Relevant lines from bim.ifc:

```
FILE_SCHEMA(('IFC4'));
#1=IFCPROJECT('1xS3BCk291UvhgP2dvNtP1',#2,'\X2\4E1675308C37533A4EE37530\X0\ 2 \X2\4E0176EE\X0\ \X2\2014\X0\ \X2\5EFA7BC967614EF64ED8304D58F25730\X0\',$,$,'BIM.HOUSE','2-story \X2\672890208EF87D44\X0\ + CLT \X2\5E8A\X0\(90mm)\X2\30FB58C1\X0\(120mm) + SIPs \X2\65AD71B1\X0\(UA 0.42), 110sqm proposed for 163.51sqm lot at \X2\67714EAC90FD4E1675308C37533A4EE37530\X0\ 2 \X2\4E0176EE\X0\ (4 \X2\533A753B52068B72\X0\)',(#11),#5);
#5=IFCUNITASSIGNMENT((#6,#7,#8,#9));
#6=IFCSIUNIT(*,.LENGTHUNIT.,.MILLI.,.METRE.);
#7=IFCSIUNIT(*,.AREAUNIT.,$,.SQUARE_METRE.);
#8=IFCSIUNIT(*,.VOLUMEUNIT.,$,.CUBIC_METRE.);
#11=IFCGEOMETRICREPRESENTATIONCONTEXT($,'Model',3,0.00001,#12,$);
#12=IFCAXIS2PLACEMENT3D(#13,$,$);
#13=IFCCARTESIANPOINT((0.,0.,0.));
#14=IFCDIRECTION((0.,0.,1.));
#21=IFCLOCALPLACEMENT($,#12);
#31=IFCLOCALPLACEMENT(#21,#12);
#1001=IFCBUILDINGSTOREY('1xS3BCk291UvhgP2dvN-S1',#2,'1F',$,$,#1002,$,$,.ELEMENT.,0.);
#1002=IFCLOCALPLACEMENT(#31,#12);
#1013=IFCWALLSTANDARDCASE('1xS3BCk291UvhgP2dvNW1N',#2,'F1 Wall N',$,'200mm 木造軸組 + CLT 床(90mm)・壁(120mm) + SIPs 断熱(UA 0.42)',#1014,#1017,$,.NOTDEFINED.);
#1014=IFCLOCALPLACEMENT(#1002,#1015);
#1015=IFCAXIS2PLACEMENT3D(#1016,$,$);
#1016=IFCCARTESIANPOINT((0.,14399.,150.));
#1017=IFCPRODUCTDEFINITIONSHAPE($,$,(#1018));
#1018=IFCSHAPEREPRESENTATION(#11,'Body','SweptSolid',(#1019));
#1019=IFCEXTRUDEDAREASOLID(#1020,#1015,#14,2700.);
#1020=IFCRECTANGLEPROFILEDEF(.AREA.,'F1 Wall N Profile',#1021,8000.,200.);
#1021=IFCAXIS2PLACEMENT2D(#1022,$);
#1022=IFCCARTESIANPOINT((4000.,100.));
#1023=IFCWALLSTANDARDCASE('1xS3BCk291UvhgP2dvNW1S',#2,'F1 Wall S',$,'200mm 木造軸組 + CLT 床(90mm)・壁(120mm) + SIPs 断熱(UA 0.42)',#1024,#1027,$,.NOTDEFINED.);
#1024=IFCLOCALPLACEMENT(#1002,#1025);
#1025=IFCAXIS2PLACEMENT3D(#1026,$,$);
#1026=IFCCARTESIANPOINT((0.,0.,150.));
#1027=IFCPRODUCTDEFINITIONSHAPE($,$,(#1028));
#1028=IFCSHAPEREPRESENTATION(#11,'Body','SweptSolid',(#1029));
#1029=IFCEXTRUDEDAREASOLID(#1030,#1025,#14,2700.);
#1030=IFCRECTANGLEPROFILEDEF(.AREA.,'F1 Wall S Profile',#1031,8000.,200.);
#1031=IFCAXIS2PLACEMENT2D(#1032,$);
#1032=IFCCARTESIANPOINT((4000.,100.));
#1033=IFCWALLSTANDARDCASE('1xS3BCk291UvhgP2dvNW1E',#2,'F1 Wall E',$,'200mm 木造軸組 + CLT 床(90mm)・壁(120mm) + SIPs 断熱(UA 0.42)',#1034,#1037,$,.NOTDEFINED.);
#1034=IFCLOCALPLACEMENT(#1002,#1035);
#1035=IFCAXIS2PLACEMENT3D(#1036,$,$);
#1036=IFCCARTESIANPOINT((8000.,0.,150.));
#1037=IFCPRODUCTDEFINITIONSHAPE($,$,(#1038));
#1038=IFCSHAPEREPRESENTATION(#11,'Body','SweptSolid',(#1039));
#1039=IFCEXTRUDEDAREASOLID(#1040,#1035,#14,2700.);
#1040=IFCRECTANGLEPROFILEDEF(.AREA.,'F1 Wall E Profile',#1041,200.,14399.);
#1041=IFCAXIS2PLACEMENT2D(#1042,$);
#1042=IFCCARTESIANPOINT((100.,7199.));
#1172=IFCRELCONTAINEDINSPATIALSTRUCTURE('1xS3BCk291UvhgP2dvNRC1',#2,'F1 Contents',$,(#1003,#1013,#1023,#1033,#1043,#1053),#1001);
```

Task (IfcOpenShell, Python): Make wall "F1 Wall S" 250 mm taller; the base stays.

```python
import ifcopenshell
import ifcopenshell.geom
import ifcopenshell.util.shape
import ifcopenshell.util.unit

model = ifcopenshell.open("bim.ifc")
unit_scale = ifcopenshell.util.unit.calculate_unit_scale(model)
settings = ifcopenshell.geom.settings()


def volume(element):
    """Net volume in cubic metres, openings subtracted."""
    shape = ifcopenshell.geom.create_shape(settings, element)
    return ifcopenshell.util.shape.get_volume(shape.geometry)


wall = model.by_id(1023)
before = volume(wall)

body = next(r for r in wall.Representation.Representations if r.RepresentationIdentifier == "Body")
solid = body.Items[0]
old_height = solid.Depth
solid.Depth += 0.25 / unit_scale
after = volume(wall)

print(f"height {old_height:g} -> {solid.Depth:g}, volume {before:.3f} -> {after:.3f} m3")

model.write("bim_updated.ifc")
```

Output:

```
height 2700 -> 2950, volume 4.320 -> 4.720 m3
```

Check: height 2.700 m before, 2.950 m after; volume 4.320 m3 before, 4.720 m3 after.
